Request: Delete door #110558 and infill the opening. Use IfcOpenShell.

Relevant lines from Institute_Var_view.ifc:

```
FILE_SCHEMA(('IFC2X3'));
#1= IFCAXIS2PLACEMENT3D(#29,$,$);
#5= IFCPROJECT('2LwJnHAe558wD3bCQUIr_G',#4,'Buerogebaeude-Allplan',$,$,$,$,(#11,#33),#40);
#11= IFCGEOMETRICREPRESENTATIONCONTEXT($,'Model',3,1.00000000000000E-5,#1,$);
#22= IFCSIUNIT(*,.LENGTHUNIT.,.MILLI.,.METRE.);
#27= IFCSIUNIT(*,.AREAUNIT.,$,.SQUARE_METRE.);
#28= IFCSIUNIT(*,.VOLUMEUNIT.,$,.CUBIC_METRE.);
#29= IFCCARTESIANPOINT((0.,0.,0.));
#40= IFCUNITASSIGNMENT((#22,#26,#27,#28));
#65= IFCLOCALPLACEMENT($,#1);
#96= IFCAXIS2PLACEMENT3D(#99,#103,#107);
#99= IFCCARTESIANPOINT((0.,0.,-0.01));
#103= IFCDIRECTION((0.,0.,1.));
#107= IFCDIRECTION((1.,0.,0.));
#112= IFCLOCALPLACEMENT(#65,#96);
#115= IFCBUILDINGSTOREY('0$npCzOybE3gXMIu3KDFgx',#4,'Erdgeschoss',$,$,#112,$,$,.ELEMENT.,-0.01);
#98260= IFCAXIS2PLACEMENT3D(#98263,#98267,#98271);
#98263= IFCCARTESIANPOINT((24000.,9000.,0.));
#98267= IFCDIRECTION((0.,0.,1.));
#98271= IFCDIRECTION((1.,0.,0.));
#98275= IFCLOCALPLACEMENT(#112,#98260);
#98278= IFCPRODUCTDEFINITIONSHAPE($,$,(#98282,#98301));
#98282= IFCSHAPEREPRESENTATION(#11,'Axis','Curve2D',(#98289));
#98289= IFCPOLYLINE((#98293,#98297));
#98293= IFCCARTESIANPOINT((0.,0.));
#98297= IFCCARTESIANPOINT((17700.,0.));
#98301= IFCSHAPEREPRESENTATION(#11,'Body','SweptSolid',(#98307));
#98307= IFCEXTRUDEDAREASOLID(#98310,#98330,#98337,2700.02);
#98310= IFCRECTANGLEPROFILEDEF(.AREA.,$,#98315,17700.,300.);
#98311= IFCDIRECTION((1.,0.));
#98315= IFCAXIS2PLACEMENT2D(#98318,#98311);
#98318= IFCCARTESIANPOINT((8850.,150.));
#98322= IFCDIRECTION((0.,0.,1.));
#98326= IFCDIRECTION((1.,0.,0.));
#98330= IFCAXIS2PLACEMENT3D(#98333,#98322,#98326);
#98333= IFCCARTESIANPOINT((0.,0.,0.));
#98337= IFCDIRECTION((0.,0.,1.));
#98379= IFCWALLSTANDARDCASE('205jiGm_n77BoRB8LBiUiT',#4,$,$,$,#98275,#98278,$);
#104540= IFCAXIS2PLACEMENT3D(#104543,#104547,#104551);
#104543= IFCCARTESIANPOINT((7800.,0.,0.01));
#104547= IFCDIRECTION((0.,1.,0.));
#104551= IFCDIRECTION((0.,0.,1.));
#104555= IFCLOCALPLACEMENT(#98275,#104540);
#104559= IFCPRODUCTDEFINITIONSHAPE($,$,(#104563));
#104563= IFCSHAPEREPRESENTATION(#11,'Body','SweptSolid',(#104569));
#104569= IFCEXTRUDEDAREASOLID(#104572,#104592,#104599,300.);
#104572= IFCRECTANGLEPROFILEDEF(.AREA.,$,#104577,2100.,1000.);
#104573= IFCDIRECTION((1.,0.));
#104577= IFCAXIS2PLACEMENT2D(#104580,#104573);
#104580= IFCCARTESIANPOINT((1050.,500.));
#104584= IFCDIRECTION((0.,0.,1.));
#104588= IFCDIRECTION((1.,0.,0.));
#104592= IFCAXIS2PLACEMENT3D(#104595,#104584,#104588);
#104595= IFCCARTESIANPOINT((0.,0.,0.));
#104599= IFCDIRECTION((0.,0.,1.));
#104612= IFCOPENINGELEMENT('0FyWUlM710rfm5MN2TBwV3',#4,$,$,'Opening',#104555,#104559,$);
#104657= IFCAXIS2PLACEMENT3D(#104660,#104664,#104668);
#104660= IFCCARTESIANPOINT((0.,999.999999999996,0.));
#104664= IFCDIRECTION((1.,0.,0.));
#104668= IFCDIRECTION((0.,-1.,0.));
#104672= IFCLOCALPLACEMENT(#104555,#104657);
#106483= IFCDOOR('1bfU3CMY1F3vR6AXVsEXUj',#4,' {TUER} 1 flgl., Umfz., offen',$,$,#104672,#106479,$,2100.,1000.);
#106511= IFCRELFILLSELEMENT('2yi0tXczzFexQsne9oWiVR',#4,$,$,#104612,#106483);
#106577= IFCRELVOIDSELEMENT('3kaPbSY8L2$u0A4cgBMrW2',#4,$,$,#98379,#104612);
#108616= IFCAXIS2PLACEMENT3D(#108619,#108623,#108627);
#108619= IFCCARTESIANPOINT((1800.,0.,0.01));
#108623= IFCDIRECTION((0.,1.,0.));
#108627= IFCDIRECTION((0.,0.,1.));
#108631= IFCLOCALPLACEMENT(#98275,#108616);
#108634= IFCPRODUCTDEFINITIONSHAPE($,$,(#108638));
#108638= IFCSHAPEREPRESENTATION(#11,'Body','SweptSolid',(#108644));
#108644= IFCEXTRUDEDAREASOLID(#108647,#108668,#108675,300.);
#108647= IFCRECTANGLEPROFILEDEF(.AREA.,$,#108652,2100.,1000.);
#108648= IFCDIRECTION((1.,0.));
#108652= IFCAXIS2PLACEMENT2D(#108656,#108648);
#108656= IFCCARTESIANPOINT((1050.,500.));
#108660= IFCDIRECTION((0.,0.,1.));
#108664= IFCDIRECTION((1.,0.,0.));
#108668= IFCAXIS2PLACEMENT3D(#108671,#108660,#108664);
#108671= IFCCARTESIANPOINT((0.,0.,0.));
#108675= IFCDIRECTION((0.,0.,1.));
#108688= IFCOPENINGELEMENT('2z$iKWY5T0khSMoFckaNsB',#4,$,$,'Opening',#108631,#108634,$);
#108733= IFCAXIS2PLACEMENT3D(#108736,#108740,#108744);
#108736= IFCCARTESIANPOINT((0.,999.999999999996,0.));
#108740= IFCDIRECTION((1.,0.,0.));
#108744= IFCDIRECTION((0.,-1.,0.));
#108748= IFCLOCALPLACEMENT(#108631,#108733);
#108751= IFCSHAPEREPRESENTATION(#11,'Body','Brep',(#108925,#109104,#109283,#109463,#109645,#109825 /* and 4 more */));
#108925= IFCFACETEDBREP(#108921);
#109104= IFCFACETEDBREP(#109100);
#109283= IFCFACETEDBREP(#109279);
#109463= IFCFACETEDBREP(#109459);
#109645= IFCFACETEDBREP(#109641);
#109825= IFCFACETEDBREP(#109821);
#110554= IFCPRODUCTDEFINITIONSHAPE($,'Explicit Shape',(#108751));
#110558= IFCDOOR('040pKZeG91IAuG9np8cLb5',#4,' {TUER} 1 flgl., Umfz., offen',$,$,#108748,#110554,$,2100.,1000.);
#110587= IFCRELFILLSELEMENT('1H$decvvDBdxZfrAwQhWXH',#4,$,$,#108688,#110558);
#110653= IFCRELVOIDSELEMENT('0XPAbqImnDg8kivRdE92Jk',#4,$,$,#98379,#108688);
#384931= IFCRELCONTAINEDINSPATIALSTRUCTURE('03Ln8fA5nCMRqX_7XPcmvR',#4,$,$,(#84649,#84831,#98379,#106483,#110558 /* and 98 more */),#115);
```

```python
import ifcopenshell
import ifcopenshell.api.feature
import ifcopenshell.api.root
import ifcopenshell.geom
import ifcopenshell.util.shape

model = ifcopenshell.open("Institute_Var_view.ifc")
settings = ifcopenshell.geom.settings()


def volume(element):
    """Net volume in cubic metres, openings subtracted."""
    shape = ifcopenshell.geom.create_shape(settings, element)
    return ifcopenshell.util.shape.get_volume(shape.geometry)


door = model.by_guid("040pKZeG91IAuG9np8cLb5")
opening = door.FillsVoids[0].RelatingOpeningElement
wall = opening.VoidsElements[0].RelatingBuildingElement
before = volume(wall)

ifcopenshell.api.root.remove_product(model, product=door)
ifcopenshell.api.feature.remove_feature(model, feature=opening)

after = volume(wall)

print(f"wall volume {before:.3f} -> {after:.3f} m3")

model.write("Institute_Var_view_rev.ifc")
```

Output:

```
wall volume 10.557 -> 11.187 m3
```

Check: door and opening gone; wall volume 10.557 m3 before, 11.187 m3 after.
